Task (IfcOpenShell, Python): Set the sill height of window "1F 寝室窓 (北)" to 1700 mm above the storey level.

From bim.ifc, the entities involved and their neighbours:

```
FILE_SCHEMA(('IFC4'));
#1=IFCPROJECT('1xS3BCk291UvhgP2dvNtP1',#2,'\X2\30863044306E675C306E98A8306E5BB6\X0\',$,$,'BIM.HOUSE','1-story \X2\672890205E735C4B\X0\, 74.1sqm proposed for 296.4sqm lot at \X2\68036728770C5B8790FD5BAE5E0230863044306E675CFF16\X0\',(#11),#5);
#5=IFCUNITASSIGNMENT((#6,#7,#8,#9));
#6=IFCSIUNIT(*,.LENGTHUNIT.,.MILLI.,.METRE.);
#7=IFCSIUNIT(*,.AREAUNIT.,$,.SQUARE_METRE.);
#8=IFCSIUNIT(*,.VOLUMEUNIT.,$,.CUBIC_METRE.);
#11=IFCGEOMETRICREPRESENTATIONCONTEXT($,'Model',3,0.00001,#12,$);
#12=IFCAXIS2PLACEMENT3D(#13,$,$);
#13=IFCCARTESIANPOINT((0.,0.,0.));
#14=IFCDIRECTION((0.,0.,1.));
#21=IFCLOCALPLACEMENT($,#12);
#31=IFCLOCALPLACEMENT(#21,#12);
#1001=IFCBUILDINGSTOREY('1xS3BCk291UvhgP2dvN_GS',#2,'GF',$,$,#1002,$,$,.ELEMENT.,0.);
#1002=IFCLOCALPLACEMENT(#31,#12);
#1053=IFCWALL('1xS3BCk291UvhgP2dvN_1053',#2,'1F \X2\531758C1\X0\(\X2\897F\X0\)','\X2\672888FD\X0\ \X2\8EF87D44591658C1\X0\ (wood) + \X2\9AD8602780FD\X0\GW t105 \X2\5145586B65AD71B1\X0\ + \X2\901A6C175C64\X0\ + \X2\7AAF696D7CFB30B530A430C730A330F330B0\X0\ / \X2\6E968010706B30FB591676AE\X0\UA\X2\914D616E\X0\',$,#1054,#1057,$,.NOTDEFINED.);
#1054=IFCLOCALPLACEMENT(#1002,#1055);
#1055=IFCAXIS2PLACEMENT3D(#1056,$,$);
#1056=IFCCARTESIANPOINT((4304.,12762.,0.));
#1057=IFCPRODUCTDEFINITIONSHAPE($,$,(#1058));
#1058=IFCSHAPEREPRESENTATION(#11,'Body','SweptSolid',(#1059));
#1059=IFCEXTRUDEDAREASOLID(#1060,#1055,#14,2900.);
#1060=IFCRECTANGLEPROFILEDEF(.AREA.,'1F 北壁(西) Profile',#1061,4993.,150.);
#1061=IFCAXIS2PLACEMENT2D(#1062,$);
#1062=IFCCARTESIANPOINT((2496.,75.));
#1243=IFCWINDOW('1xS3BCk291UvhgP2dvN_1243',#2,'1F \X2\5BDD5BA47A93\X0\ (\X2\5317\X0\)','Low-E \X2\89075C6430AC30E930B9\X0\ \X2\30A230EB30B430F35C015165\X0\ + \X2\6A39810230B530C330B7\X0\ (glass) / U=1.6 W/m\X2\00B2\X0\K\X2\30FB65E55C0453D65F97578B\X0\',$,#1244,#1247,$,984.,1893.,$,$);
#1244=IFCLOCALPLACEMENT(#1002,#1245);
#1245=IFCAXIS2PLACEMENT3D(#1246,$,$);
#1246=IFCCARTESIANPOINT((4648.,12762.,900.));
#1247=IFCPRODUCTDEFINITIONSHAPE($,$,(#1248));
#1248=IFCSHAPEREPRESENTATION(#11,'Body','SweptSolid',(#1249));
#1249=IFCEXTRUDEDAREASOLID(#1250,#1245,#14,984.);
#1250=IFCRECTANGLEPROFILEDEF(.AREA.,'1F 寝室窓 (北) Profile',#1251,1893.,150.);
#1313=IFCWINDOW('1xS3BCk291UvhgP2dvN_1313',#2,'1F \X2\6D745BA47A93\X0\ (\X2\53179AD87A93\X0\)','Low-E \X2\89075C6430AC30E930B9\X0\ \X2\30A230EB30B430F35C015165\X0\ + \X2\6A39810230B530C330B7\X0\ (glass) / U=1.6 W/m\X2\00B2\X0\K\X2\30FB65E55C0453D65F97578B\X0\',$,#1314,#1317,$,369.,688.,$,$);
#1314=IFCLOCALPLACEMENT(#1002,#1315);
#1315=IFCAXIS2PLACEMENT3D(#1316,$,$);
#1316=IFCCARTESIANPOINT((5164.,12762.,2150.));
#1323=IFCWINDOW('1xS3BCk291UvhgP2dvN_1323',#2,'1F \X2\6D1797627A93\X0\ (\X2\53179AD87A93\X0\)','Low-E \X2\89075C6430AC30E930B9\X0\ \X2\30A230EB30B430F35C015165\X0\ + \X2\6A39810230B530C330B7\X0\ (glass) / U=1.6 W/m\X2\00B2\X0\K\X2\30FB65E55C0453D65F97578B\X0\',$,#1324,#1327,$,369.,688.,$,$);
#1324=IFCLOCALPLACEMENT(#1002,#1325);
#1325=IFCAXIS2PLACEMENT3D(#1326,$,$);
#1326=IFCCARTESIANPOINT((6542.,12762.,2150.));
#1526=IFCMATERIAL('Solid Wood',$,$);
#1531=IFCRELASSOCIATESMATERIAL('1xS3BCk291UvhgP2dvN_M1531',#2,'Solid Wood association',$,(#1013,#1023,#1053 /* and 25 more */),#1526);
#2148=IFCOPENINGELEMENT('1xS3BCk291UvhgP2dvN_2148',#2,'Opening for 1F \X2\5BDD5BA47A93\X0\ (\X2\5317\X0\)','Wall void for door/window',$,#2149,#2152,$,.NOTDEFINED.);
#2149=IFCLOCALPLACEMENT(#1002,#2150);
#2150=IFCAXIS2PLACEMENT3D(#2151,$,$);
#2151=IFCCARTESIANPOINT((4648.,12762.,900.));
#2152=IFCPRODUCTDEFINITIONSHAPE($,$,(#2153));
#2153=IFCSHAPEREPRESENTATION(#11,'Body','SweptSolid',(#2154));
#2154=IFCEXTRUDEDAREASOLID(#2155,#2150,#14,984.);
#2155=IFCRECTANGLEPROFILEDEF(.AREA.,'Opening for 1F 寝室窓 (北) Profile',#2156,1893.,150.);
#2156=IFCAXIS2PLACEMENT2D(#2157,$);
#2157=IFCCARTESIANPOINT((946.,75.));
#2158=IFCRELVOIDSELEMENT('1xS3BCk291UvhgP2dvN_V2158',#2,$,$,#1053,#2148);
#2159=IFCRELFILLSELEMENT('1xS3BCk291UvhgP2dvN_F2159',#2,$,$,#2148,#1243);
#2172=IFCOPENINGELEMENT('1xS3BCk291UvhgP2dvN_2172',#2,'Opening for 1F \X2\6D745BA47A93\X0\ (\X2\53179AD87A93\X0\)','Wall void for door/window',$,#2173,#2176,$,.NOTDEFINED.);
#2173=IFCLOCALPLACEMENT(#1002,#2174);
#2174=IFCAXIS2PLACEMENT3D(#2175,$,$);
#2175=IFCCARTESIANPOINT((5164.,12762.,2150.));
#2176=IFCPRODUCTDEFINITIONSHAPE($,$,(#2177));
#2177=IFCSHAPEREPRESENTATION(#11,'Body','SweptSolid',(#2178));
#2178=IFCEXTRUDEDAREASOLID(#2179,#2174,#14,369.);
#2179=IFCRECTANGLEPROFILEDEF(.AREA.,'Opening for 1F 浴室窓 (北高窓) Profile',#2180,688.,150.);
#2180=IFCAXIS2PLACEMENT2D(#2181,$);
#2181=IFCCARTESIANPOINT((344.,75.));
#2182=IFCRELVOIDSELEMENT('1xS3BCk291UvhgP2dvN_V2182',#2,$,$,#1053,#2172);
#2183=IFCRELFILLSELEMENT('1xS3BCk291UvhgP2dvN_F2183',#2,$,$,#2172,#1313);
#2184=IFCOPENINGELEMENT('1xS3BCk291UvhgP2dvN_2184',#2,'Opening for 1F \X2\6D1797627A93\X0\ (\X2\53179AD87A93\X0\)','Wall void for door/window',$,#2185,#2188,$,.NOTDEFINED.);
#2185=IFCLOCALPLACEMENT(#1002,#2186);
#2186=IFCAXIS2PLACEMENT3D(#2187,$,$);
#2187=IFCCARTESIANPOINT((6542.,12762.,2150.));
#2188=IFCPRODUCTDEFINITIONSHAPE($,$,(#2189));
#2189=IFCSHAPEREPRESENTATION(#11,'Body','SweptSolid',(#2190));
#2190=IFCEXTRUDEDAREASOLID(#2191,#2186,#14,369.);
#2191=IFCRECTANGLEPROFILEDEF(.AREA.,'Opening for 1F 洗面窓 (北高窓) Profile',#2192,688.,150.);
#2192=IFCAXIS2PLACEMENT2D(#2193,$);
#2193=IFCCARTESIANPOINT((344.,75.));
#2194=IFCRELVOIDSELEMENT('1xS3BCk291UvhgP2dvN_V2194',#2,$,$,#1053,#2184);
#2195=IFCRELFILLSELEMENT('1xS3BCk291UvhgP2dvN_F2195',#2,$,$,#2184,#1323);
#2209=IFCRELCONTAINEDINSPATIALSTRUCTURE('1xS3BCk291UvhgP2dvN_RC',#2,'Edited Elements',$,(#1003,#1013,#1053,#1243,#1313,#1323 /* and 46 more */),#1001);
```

```python
import numpy as np
import ifcopenshell
import ifcopenshell.api.geometry
import ifcopenshell.geom
import ifcopenshell.util.element
import ifcopenshell.util.placement
import ifcopenshell.util.shape
import ifcopenshell.util.unit

model = ifcopenshell.open("bim.ifc")
unit_scale = ifcopenshell.util.unit.calculate_unit_scale(model)

window = model.by_guid("1xS3BCk291UvhgP2dvN_1243")
opening = window.FillsVoids[0].RelatingOpeningElement
storey = ifcopenshell.util.element.get_container(window, ifc_class="IfcBuildingStorey")
level = ifcopenshell.util.placement.get_local_placement(storey.ObjectPlacement)[2, 3]

# The opening's origin need not be at the sill, so measure its lowest point.
shape = ifcopenshell.geom.create_shape(ifcopenshell.geom.settings(), opening)
bottom = ifcopenshell.util.shape.get_shape_bottom_elevation(shape, shape.geometry) / unit_scale
dz = level + 1700.0 - bottom

shift = np.array([0.0, 0.0, dz])
# The window is not placed relative to its opening, so move both.
for product in (opening, window):
    matrix = ifcopenshell.util.placement.get_local_placement(product.ObjectPlacement)
    matrix[:3, 3] += shift
    ifcopenshell.api.geometry.edit_object_placement(model, product=product, matrix=matrix, is_si=False)

print(f"moved by {dz * unit_scale:+.3f} m")

model.write("bim_rev.ifc")
```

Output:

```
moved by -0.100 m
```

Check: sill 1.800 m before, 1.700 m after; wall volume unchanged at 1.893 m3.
